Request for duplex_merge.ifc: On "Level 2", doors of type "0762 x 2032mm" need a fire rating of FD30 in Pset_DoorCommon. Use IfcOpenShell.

First a look at what the model holds.

```python
import ifcopenshell
import ifcopenshell.util.element

model = ifcopenshell.open("duplex_merge.ifc")
print(model.schema)
storey = next(s for s in model.by_type("IfcBuildingStorey") if s.Name == "Level 2")
doors = [e for e in ifcopenshell.util.element.get_decomposition(storey) if e.is_a("IfcDoor")]
seen = {}
for e in doors:
    element_type = ifcopenshell.util.element.get_type(e)
    key = (element_type.Name if element_type != e and element_type else None, ifcopenshell.util.element.get_pset(e, "Pset_DoorCommon", "FireRating"))
    seen[key] = seen.get(key, 0) + 1
for (name, value), count in sorted(seen.items(), key=str):
    print(count, "x", name, "|", value)
```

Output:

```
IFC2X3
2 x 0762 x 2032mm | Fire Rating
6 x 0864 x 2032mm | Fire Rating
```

```python
import ifcopenshell
import ifcopenshell.api.pset
import ifcopenshell.util.element

model = ifcopenshell.open("duplex_merge.ifc")

storey = next(s for s in model.by_type("IfcBuildingStorey") if s.Name == "Level 2")
doors = [e for e in ifcopenshell.util.element.get_decomposition(storey) if e.is_a("IfcDoor")]

count = 0
for e in doors:
    element_type = ifcopenshell.util.element.get_type(e)
    if element_type in (None, e) or element_type.Name != "0762 x 2032mm":
        continue
    # add_pset returns the element's existing set when there is one.
    pset = ifcopenshell.api.pset.add_pset(model, product=e, name="Pset_DoorCommon")
    ifcopenshell.api.pset.edit_pset(model, pset=pset, properties={"FireRating": "FD30"})
    count += 1

print(count, "doors updated")

model.write("duplex_merge_updated.ifc")
```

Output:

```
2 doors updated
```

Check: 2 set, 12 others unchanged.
